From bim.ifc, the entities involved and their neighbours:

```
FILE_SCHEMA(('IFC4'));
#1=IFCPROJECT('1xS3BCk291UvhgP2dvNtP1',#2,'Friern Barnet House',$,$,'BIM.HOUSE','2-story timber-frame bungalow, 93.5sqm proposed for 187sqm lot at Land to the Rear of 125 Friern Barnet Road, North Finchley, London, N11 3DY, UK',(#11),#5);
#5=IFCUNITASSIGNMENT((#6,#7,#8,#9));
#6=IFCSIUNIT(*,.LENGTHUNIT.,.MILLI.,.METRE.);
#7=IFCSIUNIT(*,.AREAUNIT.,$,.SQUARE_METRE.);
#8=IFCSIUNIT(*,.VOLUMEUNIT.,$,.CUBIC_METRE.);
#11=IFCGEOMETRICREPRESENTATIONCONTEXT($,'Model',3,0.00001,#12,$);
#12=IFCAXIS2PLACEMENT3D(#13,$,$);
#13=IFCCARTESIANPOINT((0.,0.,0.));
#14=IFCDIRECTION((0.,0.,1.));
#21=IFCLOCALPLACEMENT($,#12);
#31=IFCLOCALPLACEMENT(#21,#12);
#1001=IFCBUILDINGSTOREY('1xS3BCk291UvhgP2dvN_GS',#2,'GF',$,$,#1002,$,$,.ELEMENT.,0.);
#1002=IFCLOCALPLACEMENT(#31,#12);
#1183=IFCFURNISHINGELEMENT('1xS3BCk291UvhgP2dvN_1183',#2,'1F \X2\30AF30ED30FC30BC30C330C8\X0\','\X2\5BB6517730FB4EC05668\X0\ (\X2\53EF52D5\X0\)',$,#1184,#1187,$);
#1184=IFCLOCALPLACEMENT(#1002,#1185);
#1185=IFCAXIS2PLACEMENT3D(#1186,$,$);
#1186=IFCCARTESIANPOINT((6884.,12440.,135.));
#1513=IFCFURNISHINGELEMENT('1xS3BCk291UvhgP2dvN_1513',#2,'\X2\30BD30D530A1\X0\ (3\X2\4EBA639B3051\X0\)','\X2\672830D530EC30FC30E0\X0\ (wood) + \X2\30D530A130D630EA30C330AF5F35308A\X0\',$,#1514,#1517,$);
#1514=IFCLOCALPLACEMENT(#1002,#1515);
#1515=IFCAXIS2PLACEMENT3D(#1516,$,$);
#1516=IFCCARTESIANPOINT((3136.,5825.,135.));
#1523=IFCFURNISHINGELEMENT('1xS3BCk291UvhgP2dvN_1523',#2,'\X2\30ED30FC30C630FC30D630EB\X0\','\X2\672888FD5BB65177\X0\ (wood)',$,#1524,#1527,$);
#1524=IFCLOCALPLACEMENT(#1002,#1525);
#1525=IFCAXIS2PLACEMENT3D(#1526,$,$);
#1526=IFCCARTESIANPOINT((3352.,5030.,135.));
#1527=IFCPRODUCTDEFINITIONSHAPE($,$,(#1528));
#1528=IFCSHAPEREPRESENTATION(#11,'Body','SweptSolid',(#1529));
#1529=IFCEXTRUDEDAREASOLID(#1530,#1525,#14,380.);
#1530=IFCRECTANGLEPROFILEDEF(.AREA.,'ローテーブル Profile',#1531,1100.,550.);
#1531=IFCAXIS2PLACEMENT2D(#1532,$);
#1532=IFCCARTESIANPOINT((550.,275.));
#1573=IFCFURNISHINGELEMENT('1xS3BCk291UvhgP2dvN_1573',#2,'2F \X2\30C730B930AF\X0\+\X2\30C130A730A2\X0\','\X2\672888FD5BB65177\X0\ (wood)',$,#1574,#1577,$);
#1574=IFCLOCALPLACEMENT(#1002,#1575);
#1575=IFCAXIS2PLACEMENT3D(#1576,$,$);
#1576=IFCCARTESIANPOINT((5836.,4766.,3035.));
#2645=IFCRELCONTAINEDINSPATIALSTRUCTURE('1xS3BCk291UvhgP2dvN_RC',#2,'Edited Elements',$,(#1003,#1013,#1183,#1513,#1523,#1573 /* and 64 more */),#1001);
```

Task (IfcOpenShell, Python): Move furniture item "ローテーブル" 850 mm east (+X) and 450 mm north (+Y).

```python
import ifcopenshell
import ifcopenshell.api.geometry
import ifcopenshell.util.placement
import ifcopenshell.util.unit

model = ifcopenshell.open("bim.ifc")
unit_scale = ifcopenshell.util.unit.calculate_unit_scale(model)

item = model.by_guid("1xS3BCk291UvhgP2dvN_1523")
matrix = ifcopenshell.util.placement.get_local_placement(item.ObjectPlacement)
matrix[0, 3] += 0.85 / unit_scale
matrix[1, 3] += 0.45 / unit_scale
ifcopenshell.api.geometry.edit_object_placement(model, product=item, matrix=matrix, is_si=False)

print(ifcopenshell.util.placement.get_local_placement(item.ObjectPlacement).round(3) + 0.0)

model.write("bim_edited.ifc")
```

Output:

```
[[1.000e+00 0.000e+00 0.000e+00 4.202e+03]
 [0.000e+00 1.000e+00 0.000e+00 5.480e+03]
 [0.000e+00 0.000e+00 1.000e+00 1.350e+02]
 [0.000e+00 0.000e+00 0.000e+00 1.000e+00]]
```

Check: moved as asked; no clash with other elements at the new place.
